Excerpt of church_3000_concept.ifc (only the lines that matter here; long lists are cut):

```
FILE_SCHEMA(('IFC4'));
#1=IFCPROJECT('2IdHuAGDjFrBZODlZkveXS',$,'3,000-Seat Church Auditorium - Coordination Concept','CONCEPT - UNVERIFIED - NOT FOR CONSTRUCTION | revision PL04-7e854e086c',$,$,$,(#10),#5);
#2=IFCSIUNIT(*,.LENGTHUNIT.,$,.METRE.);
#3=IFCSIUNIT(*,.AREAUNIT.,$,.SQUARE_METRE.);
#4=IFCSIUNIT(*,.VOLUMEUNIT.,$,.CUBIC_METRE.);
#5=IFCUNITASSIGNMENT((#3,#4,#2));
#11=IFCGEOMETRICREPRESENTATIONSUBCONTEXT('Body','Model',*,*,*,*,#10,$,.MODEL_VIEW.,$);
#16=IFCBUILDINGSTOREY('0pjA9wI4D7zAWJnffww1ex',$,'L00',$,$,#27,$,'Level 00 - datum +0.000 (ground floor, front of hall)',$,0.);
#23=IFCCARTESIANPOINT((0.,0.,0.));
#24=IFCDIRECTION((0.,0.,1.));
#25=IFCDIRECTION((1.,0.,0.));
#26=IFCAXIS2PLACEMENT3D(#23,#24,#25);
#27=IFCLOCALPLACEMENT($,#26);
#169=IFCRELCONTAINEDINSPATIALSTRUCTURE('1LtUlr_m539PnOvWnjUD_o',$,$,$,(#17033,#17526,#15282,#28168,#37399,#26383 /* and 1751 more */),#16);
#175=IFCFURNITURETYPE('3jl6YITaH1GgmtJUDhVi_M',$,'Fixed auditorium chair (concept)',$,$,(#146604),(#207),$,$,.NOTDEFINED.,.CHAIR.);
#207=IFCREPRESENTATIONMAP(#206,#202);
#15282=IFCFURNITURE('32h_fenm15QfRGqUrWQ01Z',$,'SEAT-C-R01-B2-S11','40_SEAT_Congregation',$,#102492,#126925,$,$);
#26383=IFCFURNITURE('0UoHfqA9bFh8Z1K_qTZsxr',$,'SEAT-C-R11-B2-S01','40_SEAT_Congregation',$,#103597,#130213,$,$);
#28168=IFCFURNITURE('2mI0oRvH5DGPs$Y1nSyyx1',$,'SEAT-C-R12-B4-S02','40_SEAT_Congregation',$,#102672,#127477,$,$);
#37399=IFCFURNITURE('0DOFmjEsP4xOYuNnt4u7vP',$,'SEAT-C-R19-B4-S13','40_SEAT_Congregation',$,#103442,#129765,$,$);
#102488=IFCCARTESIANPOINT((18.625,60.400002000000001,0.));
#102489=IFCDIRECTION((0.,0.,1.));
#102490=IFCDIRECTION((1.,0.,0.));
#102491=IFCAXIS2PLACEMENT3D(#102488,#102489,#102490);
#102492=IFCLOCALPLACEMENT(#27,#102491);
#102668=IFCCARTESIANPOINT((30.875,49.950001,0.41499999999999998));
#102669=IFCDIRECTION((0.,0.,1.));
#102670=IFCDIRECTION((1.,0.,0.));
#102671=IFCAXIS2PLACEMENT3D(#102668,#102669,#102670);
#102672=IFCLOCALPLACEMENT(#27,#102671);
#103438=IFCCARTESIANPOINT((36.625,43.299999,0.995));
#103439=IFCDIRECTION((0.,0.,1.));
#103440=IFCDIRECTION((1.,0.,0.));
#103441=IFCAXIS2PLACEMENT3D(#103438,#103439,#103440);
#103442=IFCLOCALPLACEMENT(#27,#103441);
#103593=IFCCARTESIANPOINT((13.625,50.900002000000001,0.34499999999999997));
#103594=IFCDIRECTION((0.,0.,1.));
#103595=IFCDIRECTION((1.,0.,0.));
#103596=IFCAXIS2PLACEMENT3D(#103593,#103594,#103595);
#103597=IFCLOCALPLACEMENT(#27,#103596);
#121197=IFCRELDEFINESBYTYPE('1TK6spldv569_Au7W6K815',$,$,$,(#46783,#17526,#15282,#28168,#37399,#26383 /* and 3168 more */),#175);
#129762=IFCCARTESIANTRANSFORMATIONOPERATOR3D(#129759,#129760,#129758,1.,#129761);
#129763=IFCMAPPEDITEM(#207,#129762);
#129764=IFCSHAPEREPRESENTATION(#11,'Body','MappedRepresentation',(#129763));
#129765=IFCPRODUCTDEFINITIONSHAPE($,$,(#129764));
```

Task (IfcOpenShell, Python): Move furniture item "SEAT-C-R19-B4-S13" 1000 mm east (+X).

```python
import ifcopenshell
import ifcopenshell.api.geometry
import ifcopenshell.util.placement

model = ifcopenshell.open("church_3000_concept.ifc")

item = model.by_guid("0DOFmjEsP4xOYuNnt4u7vP")
matrix = ifcopenshell.util.placement.get_local_placement(item.ObjectPlacement)
matrix[0, 3] += 1.0
ifcopenshell.api.geometry.edit_object_placement(model, product=item, matrix=matrix, is_si=False)

print(ifcopenshell.util.placement.get_local_placement(item.ObjectPlacement).round(3) + 0.0)

model.write("church_3000_concept_updated.ifc")
```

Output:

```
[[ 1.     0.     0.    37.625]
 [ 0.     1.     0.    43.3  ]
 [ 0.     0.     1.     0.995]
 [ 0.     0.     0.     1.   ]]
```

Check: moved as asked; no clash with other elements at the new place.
